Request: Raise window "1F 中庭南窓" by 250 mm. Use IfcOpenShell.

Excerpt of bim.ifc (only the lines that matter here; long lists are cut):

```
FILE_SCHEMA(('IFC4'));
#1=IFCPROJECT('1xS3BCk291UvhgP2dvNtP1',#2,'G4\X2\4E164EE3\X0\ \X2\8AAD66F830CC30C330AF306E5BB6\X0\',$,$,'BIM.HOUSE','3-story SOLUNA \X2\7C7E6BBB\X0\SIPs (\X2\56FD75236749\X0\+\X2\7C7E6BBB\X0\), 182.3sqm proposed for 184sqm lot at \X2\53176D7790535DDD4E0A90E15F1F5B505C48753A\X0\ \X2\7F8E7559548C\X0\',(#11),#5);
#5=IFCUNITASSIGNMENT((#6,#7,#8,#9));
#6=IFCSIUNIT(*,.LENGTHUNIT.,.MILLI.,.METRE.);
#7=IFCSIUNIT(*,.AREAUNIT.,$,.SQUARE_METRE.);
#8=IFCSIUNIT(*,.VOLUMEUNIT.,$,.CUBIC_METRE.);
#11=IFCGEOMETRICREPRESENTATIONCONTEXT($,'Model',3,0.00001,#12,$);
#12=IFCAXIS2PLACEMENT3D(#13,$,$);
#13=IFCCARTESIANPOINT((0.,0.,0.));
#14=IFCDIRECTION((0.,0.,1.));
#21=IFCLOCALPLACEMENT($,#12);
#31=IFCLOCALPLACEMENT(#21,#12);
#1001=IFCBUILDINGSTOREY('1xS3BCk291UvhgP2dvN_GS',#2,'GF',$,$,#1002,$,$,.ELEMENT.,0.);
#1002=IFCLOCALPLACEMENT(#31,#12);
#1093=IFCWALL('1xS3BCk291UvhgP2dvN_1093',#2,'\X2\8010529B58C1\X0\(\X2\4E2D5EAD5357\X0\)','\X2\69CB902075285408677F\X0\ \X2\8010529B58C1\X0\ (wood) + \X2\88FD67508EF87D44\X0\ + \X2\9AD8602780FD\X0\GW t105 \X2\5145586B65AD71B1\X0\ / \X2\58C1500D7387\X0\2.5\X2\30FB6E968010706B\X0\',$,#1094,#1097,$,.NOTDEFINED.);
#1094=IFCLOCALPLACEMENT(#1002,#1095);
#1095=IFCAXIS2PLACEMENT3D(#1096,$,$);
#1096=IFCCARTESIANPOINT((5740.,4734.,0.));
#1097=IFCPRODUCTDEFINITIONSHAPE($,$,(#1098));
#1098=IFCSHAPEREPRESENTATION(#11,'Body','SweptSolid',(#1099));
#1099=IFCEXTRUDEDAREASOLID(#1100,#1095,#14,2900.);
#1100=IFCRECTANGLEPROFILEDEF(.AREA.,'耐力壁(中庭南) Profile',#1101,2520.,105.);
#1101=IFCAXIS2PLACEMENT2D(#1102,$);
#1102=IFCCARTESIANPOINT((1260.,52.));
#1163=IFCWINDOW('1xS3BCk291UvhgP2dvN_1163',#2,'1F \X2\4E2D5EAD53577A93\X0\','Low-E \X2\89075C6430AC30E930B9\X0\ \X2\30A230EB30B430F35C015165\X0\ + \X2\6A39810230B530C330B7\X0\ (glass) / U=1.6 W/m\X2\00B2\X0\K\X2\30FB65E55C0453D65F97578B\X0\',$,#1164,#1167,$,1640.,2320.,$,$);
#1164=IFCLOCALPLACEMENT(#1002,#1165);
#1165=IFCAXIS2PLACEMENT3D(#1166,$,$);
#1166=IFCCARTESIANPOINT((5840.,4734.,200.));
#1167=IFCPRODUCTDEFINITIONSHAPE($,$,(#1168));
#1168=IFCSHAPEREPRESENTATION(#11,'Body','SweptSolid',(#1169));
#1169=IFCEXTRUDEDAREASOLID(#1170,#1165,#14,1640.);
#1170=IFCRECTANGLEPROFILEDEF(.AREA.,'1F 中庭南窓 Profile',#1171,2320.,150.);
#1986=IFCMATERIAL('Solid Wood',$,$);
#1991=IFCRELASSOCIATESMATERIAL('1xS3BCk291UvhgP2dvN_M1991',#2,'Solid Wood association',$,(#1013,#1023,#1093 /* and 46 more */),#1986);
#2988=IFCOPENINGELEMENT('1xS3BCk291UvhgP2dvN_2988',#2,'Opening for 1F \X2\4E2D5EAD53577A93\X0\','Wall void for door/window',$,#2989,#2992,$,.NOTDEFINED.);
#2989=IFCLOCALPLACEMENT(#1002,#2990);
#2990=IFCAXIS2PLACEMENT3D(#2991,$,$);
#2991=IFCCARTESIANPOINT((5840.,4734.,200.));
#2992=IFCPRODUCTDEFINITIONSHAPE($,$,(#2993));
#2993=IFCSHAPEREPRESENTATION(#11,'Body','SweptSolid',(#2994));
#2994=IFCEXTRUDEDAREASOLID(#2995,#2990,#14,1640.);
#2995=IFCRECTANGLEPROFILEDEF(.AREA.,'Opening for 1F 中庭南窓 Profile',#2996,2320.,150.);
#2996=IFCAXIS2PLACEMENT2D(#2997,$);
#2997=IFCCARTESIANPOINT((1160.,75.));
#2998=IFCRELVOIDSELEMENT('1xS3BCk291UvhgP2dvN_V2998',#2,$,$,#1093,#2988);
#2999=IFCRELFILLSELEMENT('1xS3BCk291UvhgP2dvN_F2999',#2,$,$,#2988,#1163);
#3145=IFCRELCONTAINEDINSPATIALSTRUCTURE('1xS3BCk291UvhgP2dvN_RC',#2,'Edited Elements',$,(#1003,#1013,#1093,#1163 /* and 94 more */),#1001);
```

```python
import numpy as np
import ifcopenshell
import ifcopenshell.api.geometry
import ifcopenshell.util.placement
import ifcopenshell.util.unit

model = ifcopenshell.open("bim.ifc")
unit_scale = ifcopenshell.util.unit.calculate_unit_scale(model)

window = model.by_guid("1xS3BCk291UvhgP2dvN_1163")
opening = window.FillsVoids[0].RelatingOpeningElement
dz = 0.25 / unit_scale

shift = np.array([0.0, 0.0, dz])
# The window is not placed relative to its opening, so move both.
for product in (opening, window):
    matrix = ifcopenshell.util.placement.get_local_placement(product.ObjectPlacement)
    matrix[:3, 3] += shift
    ifcopenshell.api.geometry.edit_object_placement(model, product=product, matrix=matrix, is_si=False)

print(f"moved by {dz * unit_scale:+.3f} m")

model.write("bim_rev.ifc")
```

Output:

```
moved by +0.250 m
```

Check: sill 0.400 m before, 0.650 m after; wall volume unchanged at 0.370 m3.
